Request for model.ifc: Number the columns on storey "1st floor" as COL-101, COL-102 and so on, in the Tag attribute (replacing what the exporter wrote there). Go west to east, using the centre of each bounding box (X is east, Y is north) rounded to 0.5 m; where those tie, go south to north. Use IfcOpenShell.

First a look at what the model holds.

```python
import ifcopenshell
import ifcopenshell.util.element
import ifcopenshell.util.placement

model = ifcopenshell.open("model.ifc")
print(model.schema)
storey = next(s for s in model.by_type("IfcBuildingStorey") if s.Name == "1st floor")
columns = [e for e in ifcopenshell.util.element.get_decomposition(storey) if e.is_a("IfcColumn")]
for e in sorted(columns, key=lambda e: e.id()):
    origin = ifcopenshell.util.placement.get_local_placement(e.ObjectPlacement)[:3, 3]
    print(e.id(), e.Tag, e.Name, origin.round(2) + 0.0, sep=" | ")
```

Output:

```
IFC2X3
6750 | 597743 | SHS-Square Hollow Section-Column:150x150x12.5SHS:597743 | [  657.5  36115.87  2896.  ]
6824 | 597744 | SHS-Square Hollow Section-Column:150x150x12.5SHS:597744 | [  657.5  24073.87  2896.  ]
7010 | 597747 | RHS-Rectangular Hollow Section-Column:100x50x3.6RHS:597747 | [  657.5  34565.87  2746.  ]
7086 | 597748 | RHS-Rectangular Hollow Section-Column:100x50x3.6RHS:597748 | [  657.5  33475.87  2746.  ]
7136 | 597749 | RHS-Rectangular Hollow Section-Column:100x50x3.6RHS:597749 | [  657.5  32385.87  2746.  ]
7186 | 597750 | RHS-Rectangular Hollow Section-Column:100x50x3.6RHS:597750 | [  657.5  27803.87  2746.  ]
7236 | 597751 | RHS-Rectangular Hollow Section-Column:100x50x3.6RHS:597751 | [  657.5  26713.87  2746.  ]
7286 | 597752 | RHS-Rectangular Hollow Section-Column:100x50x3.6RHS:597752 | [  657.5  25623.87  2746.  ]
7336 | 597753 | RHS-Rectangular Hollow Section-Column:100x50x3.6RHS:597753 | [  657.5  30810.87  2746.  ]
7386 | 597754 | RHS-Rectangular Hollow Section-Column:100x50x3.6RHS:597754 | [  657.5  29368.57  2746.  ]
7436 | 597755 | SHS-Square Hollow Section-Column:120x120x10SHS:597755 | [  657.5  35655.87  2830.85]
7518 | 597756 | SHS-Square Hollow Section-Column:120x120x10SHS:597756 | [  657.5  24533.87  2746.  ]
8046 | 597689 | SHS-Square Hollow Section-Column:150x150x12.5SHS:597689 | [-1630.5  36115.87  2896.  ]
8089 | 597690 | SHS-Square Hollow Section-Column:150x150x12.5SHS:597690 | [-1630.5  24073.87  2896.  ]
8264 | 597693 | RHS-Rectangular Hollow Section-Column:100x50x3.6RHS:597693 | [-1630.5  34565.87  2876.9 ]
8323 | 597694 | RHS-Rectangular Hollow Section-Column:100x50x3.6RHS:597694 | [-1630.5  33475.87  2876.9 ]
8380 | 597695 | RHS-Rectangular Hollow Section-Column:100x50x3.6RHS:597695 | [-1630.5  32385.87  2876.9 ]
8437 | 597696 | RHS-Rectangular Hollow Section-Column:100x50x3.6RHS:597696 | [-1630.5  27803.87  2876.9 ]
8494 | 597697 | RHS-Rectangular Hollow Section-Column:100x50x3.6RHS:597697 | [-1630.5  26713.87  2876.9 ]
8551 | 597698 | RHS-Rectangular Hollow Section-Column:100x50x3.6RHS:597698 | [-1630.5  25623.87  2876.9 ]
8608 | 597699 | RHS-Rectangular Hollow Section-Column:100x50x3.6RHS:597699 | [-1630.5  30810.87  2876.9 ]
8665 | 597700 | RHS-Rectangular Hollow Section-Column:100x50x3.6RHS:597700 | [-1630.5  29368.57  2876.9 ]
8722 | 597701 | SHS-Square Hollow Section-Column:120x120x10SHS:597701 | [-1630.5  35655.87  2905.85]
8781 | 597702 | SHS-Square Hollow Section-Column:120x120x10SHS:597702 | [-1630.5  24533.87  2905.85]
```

```python
import ifcopenshell
import ifcopenshell.geom
import ifcopenshell.util.element
import ifcopenshell.util.shape

model = ifcopenshell.open("model.ifc")
settings = ifcopenshell.geom.settings()
settings.set("use-world-coords", True)


def centre(element):
    shape = ifcopenshell.geom.create_shape(settings, element)
    return ifcopenshell.util.shape.get_bbox_centroid(shape.geometry)


storey = next(s for s in model.by_type("IfcBuildingStorey") if s.Name == "1st floor")
columns = [e for e in ifcopenshell.util.element.get_decomposition(storey) if e.is_a("IfcColumn")]

# Insertion points can sit at a corner or the storey origin, so sort by the geometry (in metres).
centres = {e: centre(e) for e in columns}
columns.sort(key=lambda e: (round(centres[e][0] / 0.5), centres[e][1]))

for i, e in enumerate(columns, start=1):
    number = f"COL-1{i:02d}"
    e.Tag = number
    print(e.id(), number)

model.write("model_rev.ifc")
```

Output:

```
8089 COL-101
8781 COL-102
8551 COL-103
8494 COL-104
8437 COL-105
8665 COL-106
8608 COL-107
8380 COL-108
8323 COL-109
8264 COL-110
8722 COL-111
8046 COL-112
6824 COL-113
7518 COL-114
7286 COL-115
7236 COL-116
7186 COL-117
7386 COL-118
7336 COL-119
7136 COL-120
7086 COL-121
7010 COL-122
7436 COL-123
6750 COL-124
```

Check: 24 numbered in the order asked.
